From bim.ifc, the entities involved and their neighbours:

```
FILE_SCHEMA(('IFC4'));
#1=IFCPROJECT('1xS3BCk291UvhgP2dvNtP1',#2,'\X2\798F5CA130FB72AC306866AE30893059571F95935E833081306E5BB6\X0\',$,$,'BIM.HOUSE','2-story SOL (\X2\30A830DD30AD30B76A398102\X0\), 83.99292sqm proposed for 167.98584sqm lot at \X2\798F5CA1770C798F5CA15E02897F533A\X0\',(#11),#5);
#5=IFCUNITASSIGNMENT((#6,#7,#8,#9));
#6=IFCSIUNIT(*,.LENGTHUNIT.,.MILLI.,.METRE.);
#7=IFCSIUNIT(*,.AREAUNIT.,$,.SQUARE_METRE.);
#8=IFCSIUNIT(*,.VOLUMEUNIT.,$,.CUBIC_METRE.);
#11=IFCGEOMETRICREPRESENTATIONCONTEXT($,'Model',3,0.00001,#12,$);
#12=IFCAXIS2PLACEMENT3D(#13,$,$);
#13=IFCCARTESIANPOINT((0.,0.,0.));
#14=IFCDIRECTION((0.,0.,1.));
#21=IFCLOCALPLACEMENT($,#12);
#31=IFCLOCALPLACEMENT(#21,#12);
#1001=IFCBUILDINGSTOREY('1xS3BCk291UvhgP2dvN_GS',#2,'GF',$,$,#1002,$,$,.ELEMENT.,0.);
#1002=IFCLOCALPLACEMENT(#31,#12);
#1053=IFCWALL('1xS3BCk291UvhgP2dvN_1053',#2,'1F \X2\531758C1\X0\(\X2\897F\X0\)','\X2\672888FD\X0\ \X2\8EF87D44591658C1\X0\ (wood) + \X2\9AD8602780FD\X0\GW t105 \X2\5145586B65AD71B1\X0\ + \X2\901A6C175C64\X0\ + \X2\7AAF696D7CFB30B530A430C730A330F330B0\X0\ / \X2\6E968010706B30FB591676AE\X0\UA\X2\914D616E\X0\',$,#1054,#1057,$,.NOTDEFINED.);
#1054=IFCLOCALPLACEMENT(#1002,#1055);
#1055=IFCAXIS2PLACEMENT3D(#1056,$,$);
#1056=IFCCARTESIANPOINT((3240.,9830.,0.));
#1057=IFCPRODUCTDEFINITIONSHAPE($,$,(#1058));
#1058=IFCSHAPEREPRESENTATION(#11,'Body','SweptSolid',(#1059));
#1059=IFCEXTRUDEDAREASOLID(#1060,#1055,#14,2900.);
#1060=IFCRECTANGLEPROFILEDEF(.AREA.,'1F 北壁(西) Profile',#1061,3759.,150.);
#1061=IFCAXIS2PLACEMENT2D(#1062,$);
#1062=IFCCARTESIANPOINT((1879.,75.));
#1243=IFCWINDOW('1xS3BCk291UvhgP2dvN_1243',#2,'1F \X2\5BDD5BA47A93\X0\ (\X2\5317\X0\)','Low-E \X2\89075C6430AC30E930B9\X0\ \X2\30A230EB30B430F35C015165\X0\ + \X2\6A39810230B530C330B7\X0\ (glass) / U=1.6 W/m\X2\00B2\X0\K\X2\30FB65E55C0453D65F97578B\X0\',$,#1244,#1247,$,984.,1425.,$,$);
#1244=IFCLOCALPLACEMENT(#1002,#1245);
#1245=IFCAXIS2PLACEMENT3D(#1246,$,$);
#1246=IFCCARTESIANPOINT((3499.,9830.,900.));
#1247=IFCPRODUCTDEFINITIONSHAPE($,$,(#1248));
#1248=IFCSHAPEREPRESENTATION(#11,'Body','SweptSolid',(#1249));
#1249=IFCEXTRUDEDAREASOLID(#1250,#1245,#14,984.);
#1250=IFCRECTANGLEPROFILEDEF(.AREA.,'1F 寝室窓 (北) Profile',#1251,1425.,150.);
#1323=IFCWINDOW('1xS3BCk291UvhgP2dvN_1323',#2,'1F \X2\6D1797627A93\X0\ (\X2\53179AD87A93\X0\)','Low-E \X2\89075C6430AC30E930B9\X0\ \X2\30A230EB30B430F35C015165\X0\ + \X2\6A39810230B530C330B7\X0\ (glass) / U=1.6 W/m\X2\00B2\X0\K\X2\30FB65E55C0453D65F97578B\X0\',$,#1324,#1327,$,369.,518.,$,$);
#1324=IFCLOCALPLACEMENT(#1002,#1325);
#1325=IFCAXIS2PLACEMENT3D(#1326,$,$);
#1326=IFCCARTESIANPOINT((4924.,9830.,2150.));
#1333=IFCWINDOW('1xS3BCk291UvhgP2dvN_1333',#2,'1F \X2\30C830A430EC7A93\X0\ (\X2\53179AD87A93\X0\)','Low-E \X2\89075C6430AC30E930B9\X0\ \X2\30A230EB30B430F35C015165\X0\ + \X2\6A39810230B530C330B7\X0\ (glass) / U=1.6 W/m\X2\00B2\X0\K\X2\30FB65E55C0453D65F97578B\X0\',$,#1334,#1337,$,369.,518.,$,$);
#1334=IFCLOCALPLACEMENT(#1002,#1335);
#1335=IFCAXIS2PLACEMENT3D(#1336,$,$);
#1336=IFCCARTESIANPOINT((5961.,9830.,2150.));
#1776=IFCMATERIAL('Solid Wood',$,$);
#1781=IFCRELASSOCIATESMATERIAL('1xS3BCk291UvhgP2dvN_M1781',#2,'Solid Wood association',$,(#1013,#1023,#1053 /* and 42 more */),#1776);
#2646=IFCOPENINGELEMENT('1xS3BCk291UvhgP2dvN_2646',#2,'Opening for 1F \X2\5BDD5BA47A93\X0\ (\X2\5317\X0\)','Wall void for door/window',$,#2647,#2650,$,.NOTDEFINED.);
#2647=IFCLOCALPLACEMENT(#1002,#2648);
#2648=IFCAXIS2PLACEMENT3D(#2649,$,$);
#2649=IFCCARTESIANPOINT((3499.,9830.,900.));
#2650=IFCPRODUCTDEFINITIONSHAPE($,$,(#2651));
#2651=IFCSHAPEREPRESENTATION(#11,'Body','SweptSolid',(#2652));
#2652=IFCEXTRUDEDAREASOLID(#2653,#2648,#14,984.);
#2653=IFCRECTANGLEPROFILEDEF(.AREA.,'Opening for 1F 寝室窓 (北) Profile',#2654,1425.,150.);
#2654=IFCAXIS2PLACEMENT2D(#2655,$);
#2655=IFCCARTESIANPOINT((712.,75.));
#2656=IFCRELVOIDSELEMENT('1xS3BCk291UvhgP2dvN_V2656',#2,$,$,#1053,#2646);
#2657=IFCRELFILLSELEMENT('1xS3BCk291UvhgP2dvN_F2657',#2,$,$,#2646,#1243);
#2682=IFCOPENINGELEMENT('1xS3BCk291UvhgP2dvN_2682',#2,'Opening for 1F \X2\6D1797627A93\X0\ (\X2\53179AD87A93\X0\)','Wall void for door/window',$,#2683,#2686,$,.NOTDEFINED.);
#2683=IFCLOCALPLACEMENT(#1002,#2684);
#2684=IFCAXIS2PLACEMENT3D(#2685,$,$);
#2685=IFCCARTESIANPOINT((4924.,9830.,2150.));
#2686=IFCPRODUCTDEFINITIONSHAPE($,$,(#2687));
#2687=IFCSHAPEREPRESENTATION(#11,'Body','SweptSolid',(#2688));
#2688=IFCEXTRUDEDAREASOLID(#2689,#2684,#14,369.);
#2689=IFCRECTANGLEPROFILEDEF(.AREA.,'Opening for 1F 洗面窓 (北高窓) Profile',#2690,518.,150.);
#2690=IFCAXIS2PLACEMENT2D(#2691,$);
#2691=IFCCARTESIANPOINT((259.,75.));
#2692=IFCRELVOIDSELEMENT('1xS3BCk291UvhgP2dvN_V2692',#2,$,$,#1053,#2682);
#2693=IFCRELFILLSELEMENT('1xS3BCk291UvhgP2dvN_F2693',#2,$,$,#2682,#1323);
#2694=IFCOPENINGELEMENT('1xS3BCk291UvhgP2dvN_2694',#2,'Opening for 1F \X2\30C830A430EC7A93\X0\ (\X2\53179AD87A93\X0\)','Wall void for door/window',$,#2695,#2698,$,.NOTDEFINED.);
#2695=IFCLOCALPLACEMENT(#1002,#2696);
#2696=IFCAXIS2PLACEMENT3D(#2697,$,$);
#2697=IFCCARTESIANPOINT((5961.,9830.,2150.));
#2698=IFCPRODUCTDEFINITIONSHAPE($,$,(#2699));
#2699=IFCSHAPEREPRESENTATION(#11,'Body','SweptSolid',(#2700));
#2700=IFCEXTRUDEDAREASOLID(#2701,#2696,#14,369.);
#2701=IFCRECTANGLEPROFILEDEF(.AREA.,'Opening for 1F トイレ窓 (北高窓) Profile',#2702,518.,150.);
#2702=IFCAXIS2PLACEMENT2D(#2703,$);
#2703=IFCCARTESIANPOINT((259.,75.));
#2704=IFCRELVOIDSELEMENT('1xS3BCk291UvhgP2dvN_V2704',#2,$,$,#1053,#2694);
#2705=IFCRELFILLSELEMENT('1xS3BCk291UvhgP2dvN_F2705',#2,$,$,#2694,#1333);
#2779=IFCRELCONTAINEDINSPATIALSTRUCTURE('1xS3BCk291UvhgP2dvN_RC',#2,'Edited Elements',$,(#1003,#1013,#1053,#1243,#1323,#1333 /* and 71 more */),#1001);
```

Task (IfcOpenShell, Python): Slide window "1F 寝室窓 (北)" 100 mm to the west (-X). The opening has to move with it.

```python
import ifcopenshell
import ifcopenshell.api.geometry
import ifcopenshell.util.placement
import ifcopenshell.util.unit

model = ifcopenshell.open("bim.ifc")
unit_scale = ifcopenshell.util.unit.calculate_unit_scale(model)

window = model.by_guid("1xS3BCk291UvhgP2dvN_1243")
opening = window.FillsVoids[0].RelatingOpeningElement
wall = opening.VoidsElements[0].RelatingBuildingElement

wall_matrix = ifcopenshell.util.placement.get_local_placement(wall.ObjectPlacement)
shift = wall_matrix[:3, 0] * -0.1 / unit_scale
before = ifcopenshell.util.placement.get_local_placement(window.ObjectPlacement)[:3, 3].copy()

# The window is not placed relative to its opening, so move both.
for product in (opening, window):
    matrix = ifcopenshell.util.placement.get_local_placement(product.ObjectPlacement)
    matrix[:3, 3] += shift
    ifcopenshell.api.geometry.edit_object_placement(model, product=product, matrix=matrix, is_si=False)

after = ifcopenshell.util.placement.get_local_placement(window.ObjectPlacement)[:3, 3]
print("window moved by", (after - before).round(3) + 0.0)

model.write("bim_rev.ifc")
```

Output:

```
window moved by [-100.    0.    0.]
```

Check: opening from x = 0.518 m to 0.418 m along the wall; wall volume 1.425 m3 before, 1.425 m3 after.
